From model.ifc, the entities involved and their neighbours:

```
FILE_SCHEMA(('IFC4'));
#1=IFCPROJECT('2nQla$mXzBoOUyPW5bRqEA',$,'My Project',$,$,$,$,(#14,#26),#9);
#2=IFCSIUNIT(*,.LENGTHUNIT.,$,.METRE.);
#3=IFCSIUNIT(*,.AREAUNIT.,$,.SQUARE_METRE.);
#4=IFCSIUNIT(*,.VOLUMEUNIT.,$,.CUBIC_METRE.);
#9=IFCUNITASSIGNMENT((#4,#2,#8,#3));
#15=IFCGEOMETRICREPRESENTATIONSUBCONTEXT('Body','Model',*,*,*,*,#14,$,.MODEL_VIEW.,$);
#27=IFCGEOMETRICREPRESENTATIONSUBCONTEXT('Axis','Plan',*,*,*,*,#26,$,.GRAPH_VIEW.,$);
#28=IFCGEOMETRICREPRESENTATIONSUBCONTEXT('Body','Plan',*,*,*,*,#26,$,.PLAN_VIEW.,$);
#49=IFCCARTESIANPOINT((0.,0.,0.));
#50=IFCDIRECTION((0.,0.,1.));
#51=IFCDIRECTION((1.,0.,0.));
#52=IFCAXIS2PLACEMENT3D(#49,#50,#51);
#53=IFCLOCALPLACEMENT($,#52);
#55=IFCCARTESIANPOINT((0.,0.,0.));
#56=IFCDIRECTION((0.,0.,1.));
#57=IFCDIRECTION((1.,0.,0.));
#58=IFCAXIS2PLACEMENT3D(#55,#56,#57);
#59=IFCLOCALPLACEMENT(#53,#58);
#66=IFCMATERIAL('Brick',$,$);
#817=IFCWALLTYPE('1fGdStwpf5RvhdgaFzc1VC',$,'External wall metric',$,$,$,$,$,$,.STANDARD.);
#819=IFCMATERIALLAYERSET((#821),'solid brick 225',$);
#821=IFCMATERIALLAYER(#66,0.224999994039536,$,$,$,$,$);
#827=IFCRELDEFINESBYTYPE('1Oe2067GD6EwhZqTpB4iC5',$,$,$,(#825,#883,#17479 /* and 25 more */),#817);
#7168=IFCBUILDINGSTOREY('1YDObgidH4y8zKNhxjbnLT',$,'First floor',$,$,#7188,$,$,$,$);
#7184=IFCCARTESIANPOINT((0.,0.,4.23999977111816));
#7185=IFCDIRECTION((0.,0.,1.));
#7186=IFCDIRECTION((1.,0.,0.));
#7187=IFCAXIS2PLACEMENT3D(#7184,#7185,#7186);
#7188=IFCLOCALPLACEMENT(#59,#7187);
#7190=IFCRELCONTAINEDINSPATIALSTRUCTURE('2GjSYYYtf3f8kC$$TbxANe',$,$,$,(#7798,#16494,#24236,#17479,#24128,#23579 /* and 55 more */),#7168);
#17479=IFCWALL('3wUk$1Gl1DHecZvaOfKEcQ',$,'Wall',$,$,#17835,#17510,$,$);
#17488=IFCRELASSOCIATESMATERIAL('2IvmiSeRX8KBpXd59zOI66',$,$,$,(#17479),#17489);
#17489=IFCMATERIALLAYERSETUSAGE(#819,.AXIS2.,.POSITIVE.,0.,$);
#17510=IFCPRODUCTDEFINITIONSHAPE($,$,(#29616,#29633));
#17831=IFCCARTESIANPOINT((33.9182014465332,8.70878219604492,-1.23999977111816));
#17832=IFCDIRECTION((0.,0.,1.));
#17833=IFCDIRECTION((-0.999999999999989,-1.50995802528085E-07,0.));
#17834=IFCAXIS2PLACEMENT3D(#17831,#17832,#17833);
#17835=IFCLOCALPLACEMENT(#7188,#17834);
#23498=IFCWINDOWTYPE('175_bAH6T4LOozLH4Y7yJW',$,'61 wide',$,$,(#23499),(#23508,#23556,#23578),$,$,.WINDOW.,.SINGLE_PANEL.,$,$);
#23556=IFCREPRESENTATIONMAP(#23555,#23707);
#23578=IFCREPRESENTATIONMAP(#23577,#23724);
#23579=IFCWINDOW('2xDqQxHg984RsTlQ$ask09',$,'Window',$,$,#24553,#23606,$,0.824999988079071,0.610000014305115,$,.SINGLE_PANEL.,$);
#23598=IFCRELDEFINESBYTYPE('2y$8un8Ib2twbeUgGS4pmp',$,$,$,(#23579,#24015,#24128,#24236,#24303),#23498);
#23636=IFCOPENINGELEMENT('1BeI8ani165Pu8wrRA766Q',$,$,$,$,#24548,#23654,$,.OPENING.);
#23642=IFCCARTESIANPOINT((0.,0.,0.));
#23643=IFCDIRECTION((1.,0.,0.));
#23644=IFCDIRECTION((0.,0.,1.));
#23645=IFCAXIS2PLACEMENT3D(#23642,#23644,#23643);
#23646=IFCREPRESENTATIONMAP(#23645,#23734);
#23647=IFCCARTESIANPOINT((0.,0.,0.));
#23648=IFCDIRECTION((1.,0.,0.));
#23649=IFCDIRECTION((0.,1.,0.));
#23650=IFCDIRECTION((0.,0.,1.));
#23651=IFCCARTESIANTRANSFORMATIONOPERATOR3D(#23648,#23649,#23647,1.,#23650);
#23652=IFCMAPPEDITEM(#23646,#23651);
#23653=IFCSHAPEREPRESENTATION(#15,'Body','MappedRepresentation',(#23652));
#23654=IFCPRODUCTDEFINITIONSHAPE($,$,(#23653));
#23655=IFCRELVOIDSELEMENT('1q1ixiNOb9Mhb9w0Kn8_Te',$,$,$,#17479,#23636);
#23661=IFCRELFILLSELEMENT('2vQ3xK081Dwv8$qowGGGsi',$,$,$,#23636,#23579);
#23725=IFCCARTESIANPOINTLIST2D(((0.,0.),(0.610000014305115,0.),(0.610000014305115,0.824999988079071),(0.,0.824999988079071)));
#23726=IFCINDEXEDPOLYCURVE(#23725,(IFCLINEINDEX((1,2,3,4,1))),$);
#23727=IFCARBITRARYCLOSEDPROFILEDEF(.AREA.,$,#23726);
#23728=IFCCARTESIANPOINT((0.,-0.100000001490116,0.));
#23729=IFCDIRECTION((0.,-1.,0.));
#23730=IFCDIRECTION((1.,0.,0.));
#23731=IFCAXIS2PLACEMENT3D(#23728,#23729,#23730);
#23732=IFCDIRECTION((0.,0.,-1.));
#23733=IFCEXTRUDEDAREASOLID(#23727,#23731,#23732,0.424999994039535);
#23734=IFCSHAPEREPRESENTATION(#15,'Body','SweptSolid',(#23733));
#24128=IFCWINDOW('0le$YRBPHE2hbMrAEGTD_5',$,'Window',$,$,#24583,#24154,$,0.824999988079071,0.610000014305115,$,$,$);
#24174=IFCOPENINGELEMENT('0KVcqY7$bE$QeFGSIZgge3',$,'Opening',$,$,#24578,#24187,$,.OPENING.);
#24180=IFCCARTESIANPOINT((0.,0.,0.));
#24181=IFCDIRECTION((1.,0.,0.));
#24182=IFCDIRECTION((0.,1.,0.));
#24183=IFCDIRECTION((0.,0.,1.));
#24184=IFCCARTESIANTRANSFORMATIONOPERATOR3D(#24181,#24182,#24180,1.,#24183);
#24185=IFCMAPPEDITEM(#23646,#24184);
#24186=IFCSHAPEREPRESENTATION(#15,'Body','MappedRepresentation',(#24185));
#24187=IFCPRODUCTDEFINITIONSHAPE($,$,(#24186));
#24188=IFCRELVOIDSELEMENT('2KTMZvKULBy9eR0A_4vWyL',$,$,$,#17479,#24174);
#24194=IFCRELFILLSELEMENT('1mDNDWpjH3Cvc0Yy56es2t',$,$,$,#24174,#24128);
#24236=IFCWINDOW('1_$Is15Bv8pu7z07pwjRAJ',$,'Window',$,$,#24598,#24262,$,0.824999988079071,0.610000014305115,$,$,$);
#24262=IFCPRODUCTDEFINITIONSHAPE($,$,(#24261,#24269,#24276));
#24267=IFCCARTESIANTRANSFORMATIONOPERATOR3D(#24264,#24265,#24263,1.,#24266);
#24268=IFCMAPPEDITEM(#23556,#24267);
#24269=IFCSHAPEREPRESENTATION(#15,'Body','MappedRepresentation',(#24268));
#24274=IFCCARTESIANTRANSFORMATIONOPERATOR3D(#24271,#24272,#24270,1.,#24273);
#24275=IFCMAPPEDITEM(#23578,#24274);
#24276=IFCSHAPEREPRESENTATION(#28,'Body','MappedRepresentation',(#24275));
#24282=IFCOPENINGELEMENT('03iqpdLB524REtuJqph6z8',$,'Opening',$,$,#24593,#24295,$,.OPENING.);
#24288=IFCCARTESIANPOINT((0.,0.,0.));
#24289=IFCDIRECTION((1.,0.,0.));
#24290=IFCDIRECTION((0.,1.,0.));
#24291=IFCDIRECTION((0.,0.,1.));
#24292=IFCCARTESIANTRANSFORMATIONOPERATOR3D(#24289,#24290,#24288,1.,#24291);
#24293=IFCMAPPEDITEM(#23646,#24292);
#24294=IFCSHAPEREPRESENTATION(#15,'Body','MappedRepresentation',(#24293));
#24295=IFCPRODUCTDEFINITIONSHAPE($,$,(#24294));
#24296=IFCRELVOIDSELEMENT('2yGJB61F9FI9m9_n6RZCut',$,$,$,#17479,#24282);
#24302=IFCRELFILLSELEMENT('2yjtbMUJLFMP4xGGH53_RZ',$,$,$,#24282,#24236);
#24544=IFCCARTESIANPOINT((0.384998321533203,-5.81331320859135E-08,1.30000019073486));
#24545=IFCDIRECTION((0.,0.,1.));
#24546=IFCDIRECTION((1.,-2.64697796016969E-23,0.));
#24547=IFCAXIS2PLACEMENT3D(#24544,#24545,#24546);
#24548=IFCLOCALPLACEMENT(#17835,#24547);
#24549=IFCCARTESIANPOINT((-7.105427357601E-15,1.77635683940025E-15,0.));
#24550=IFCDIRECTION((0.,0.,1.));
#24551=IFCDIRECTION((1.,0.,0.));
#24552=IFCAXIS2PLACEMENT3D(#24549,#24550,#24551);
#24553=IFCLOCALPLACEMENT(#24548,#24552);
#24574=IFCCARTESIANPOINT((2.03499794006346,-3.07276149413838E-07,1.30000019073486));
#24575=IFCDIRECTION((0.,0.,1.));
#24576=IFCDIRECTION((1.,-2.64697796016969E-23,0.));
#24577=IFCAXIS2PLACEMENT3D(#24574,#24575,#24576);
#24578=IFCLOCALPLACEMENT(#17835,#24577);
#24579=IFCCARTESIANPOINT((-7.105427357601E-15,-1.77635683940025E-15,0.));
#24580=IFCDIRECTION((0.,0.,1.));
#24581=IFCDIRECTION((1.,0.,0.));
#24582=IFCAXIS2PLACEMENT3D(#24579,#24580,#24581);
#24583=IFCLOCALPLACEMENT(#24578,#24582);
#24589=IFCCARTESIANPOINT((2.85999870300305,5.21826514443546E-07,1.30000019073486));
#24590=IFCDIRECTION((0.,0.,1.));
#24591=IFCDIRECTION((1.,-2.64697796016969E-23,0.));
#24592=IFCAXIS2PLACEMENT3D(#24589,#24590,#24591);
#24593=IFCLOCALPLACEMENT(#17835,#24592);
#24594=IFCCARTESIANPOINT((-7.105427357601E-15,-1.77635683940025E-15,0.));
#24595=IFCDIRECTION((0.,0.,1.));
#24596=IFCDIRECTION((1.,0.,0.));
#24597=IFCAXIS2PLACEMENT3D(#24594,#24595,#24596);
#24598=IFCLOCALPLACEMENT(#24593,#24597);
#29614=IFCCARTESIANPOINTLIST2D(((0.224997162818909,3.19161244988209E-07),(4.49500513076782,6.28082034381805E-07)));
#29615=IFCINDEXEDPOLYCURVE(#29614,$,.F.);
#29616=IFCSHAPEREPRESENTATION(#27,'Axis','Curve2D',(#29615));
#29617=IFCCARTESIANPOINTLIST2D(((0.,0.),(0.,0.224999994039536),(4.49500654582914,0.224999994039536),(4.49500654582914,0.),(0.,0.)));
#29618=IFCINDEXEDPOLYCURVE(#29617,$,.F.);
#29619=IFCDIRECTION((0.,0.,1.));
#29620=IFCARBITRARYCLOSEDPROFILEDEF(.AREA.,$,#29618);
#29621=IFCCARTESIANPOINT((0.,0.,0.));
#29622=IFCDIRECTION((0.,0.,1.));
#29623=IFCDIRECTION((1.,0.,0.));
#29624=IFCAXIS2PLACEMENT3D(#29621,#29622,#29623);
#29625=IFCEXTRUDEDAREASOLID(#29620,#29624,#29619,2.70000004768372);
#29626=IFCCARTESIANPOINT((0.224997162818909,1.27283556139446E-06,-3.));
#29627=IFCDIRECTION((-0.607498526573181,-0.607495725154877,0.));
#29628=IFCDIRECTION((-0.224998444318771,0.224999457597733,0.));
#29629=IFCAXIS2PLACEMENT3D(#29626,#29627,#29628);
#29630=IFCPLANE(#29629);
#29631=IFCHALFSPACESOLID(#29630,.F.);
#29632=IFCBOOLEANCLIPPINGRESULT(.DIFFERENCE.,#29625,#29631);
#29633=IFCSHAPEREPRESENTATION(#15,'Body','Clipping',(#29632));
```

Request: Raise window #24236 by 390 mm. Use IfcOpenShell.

```python
import numpy as np
import ifcopenshell
import ifcopenshell.api.geometry
import ifcopenshell.util.placement
import ifcopenshell.util.unit

model = ifcopenshell.open("model.ifc")
unit_scale = ifcopenshell.util.unit.calculate_unit_scale(model)

window = model.by_guid("1_$Is15Bv8pu7z07pwjRAJ")
opening = window.FillsVoids[0].RelatingOpeningElement
dz = 0.39 / unit_scale

shift = np.array([0.0, 0.0, dz])
# The window is placed relative to its opening, so it follows when the opening moves.
matrix = ifcopenshell.util.placement.get_local_placement(opening.ObjectPlacement)
matrix[:3, 3] += shift
ifcopenshell.api.geometry.edit_object_placement(
    model, product=opening, matrix=matrix, is_si=False, should_transform_children=True
)

print(f"moved by {dz * unit_scale:+.3f} m")

model.write("model-out.ifc")
```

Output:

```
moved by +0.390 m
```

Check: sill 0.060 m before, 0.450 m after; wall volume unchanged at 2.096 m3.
